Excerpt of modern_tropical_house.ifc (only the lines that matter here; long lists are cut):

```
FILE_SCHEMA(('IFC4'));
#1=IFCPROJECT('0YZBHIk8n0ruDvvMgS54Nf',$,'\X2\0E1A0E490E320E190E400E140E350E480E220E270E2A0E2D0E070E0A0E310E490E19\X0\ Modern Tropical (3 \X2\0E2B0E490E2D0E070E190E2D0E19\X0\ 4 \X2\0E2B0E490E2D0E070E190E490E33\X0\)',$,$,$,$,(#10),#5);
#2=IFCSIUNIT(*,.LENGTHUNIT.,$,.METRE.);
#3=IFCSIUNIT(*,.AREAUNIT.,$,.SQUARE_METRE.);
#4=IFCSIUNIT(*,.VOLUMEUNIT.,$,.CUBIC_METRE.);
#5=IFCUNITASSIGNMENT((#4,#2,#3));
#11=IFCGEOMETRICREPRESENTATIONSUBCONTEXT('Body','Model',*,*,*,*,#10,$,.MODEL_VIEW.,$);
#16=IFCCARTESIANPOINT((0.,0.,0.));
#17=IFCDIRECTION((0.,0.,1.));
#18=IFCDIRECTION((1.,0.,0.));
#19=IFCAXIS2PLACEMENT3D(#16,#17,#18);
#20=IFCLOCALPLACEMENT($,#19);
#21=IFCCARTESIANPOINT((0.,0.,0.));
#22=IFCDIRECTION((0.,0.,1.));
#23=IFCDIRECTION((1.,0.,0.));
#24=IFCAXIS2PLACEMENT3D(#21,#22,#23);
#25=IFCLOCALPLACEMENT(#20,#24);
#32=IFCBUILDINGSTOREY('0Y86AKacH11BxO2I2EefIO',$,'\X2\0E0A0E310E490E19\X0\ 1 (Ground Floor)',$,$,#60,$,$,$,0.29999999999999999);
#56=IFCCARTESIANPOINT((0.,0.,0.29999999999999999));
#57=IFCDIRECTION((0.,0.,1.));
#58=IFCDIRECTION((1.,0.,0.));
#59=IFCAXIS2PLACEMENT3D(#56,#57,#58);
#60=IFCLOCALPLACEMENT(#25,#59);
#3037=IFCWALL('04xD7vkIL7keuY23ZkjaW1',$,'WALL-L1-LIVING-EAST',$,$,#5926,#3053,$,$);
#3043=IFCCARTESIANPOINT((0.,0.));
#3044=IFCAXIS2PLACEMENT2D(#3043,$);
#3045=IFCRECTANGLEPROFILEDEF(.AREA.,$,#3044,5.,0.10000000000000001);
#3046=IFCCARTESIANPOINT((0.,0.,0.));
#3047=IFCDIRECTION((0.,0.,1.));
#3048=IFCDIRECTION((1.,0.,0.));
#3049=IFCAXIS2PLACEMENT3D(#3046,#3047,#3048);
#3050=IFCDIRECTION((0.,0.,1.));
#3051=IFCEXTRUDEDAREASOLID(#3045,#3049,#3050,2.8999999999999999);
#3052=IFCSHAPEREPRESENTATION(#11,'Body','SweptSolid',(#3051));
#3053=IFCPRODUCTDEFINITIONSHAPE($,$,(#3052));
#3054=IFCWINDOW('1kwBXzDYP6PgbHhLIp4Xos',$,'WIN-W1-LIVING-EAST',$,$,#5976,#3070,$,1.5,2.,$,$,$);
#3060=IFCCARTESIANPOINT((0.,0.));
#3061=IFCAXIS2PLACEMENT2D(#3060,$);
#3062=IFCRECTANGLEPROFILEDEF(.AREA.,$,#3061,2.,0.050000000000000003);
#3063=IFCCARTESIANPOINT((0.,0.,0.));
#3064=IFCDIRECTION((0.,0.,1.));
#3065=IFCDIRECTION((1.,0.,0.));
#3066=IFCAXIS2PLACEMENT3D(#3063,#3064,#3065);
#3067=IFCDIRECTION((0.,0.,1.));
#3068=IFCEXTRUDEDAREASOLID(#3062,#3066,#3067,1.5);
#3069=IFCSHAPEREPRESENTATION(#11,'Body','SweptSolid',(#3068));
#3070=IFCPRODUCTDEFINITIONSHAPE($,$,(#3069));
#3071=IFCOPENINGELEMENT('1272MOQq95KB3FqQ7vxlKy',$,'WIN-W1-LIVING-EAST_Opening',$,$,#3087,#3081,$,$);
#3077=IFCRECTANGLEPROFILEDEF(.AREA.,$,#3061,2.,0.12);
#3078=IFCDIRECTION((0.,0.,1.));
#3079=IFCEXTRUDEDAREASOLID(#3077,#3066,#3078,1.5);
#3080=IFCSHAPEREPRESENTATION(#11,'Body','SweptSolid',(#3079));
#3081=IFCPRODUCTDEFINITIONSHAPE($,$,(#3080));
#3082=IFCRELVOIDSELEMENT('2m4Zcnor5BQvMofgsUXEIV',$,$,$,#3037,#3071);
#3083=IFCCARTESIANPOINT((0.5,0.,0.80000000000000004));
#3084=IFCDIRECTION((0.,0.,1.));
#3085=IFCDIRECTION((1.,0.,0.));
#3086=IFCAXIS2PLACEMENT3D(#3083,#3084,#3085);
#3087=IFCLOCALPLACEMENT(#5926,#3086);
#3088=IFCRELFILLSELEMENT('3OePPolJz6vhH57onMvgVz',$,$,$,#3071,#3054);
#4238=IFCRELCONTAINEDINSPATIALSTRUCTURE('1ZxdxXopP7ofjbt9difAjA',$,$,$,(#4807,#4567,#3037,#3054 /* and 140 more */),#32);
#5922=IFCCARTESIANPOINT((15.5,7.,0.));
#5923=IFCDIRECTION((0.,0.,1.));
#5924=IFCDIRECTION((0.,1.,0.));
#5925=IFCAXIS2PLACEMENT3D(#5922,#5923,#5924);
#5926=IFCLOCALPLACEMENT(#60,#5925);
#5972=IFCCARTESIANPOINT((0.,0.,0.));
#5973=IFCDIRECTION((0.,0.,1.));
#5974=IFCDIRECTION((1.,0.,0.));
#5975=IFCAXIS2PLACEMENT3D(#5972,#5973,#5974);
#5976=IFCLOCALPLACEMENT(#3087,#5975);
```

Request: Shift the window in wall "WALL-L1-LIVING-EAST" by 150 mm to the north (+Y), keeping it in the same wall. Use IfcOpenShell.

```python
import ifcopenshell
import ifcopenshell.api.geometry
import ifcopenshell.util.placement
import ifcopenshell.util.unit

model = ifcopenshell.open("modern_tropical_house.ifc")
unit_scale = ifcopenshell.util.unit.calculate_unit_scale(model)

window = model.by_id(3054)
opening = window.FillsVoids[0].RelatingOpeningElement
wall = opening.VoidsElements[0].RelatingBuildingElement

wall_matrix = ifcopenshell.util.placement.get_local_placement(wall.ObjectPlacement)
shift = wall_matrix[:3, 0] * 0.15 / unit_scale
before = ifcopenshell.util.placement.get_local_placement(window.ObjectPlacement)[:3, 3].copy()

# The window is placed relative to its opening, so it follows when the opening moves.
matrix = ifcopenshell.util.placement.get_local_placement(opening.ObjectPlacement)
matrix[:3, 3] += shift
ifcopenshell.api.geometry.edit_object_placement(
    model, product=opening, matrix=matrix, is_si=False, should_transform_children=True
)

after = ifcopenshell.util.placement.get_local_placement(window.ObjectPlacement)[:3, 3]
print("window moved by", (after - before).round(3) + 0.0)

model.write("modern_tropical_house_updated.ifc")
```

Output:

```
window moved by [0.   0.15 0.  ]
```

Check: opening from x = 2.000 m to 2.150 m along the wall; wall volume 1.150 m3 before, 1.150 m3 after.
